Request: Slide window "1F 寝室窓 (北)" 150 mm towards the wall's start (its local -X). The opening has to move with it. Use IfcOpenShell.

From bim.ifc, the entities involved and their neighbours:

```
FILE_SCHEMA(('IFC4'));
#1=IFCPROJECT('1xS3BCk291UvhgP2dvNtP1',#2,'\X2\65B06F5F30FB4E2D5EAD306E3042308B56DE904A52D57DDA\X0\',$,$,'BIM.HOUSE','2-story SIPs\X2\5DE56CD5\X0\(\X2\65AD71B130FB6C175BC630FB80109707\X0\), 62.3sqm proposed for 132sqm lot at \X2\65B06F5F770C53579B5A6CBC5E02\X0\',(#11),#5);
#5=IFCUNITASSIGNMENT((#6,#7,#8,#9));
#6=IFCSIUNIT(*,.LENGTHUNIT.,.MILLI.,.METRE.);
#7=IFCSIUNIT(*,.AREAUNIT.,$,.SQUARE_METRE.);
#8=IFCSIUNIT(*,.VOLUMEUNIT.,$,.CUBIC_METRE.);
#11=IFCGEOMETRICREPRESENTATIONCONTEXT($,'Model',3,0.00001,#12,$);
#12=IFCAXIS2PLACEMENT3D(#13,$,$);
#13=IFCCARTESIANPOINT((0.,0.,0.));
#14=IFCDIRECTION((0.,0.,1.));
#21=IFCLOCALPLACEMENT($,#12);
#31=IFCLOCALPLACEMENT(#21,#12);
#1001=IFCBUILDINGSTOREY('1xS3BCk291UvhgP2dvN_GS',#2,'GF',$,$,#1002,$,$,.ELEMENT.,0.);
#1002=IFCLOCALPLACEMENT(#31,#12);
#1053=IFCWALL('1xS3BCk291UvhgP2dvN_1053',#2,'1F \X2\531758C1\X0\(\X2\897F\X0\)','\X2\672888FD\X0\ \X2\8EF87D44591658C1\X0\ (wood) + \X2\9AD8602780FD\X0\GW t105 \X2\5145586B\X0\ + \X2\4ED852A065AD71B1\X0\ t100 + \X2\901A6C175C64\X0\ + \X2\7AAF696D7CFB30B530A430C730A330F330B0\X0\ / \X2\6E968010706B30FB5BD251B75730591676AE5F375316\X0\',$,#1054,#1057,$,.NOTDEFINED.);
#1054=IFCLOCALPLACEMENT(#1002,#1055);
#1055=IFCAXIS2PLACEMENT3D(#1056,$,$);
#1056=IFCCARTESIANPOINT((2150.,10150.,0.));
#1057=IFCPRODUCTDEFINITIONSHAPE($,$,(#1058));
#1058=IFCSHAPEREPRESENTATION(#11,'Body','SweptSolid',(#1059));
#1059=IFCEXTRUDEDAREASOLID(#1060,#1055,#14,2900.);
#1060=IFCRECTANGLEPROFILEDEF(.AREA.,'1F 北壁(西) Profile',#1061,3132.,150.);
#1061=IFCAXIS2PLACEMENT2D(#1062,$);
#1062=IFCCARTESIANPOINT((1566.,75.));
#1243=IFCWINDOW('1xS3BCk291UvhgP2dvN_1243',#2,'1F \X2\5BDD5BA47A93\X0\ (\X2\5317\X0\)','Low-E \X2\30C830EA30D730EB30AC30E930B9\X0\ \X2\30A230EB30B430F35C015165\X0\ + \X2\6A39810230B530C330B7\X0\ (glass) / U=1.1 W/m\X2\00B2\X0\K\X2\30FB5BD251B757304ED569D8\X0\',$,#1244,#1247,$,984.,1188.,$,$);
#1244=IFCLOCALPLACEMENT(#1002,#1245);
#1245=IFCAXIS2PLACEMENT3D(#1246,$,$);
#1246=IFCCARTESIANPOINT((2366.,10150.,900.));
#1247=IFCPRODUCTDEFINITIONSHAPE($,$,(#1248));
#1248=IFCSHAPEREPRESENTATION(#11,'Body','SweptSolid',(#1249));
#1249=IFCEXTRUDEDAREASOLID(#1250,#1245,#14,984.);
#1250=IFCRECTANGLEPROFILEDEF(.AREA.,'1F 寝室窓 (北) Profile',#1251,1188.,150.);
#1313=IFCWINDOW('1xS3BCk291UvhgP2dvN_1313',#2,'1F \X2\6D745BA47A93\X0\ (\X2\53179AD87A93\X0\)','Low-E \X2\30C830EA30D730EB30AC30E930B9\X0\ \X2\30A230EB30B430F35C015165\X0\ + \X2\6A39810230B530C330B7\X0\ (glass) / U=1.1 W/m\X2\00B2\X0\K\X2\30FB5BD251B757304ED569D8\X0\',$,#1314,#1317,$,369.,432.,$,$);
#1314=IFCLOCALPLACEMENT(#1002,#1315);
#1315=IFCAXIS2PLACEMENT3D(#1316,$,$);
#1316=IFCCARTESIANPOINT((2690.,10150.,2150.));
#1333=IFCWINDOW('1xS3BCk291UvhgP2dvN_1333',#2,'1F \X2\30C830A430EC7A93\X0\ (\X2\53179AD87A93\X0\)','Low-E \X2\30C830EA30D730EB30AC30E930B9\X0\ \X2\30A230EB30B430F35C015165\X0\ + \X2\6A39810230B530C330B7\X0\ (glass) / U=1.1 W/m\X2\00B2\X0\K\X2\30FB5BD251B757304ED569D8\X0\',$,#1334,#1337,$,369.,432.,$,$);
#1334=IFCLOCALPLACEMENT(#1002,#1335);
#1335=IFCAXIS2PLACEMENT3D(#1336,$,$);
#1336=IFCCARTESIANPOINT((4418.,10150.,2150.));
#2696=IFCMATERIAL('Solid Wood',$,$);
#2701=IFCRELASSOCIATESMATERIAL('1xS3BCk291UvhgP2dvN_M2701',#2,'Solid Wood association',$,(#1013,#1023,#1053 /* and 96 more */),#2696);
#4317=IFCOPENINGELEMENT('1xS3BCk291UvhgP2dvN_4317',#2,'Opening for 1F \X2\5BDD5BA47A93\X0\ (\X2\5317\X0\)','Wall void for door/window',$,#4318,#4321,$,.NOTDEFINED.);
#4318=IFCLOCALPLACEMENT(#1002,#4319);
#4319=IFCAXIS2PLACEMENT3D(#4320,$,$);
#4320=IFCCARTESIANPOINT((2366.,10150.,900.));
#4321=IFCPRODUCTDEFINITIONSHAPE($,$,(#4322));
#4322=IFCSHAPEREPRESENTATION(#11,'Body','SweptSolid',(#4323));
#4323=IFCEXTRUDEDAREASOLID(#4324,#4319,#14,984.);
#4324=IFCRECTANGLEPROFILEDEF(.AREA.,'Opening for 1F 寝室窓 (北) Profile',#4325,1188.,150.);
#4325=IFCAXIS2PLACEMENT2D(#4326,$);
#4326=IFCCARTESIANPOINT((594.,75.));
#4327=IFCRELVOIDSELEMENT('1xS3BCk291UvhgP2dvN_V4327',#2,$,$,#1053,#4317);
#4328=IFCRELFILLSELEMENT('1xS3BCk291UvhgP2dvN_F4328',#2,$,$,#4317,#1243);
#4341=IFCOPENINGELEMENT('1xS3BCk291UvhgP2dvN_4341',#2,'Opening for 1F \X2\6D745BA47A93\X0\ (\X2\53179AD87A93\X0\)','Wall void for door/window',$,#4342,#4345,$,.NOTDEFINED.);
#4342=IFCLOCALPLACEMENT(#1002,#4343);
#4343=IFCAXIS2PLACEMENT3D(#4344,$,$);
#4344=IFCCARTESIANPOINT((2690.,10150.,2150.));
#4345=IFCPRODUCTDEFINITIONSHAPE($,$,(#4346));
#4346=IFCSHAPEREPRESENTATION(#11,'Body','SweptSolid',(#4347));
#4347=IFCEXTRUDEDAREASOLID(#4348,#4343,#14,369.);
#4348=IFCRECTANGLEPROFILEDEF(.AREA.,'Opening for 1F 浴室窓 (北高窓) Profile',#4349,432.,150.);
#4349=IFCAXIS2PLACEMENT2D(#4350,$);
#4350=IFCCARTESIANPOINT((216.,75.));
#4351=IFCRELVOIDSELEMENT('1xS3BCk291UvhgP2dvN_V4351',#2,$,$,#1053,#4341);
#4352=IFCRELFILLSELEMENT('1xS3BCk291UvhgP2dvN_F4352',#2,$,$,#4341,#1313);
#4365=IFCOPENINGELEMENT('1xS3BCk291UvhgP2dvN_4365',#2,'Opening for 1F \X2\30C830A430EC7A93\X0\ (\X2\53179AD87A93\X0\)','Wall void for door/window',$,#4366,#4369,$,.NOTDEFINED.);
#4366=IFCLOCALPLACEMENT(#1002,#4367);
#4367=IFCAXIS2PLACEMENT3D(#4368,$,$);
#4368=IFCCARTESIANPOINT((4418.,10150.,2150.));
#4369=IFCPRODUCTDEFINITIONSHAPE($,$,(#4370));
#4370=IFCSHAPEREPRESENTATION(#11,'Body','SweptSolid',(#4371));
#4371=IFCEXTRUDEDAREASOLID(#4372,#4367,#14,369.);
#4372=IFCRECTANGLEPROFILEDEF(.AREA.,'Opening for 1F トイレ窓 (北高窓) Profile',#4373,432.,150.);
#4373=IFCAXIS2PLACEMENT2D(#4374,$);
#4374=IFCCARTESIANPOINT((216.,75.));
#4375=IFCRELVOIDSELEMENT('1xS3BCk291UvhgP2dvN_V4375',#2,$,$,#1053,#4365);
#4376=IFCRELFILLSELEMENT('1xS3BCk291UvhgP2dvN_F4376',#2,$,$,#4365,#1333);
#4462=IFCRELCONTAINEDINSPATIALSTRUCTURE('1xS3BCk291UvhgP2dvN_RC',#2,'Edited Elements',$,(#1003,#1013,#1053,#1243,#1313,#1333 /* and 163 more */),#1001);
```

```python
import ifcopenshell
import ifcopenshell.api.geometry
import ifcopenshell.util.placement

model = ifcopenshell.open("bim.ifc")

window = model.by_guid("1xS3BCk291UvhgP2dvN_1243")
opening = window.FillsVoids[0].RelatingOpeningElement
wall = opening.VoidsElements[0].RelatingBuildingElement

wall_matrix = ifcopenshell.util.placement.get_local_placement(wall.ObjectPlacement)
shift = wall_matrix[:3, 0] * -150.0
before = ifcopenshell.util.placement.get_local_placement(window.ObjectPlacement)[:3, 3].copy()

# The window is not placed relative to its opening, so move both.
for product in (opening, window):
    matrix = ifcopenshell.util.placement.get_local_placement(product.ObjectPlacement)
    matrix[:3, 3] += shift
    ifcopenshell.api.geometry.edit_object_placement(model, product=product, matrix=matrix, is_si=False)

after = ifcopenshell.util.placement.get_local_placement(window.ObjectPlacement)[:3, 3]
print("window moved by", (after - before).round(3) + 0.0)

model.write("bim_v2.ifc")
```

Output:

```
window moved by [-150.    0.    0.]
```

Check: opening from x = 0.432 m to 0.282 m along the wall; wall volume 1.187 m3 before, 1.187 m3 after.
